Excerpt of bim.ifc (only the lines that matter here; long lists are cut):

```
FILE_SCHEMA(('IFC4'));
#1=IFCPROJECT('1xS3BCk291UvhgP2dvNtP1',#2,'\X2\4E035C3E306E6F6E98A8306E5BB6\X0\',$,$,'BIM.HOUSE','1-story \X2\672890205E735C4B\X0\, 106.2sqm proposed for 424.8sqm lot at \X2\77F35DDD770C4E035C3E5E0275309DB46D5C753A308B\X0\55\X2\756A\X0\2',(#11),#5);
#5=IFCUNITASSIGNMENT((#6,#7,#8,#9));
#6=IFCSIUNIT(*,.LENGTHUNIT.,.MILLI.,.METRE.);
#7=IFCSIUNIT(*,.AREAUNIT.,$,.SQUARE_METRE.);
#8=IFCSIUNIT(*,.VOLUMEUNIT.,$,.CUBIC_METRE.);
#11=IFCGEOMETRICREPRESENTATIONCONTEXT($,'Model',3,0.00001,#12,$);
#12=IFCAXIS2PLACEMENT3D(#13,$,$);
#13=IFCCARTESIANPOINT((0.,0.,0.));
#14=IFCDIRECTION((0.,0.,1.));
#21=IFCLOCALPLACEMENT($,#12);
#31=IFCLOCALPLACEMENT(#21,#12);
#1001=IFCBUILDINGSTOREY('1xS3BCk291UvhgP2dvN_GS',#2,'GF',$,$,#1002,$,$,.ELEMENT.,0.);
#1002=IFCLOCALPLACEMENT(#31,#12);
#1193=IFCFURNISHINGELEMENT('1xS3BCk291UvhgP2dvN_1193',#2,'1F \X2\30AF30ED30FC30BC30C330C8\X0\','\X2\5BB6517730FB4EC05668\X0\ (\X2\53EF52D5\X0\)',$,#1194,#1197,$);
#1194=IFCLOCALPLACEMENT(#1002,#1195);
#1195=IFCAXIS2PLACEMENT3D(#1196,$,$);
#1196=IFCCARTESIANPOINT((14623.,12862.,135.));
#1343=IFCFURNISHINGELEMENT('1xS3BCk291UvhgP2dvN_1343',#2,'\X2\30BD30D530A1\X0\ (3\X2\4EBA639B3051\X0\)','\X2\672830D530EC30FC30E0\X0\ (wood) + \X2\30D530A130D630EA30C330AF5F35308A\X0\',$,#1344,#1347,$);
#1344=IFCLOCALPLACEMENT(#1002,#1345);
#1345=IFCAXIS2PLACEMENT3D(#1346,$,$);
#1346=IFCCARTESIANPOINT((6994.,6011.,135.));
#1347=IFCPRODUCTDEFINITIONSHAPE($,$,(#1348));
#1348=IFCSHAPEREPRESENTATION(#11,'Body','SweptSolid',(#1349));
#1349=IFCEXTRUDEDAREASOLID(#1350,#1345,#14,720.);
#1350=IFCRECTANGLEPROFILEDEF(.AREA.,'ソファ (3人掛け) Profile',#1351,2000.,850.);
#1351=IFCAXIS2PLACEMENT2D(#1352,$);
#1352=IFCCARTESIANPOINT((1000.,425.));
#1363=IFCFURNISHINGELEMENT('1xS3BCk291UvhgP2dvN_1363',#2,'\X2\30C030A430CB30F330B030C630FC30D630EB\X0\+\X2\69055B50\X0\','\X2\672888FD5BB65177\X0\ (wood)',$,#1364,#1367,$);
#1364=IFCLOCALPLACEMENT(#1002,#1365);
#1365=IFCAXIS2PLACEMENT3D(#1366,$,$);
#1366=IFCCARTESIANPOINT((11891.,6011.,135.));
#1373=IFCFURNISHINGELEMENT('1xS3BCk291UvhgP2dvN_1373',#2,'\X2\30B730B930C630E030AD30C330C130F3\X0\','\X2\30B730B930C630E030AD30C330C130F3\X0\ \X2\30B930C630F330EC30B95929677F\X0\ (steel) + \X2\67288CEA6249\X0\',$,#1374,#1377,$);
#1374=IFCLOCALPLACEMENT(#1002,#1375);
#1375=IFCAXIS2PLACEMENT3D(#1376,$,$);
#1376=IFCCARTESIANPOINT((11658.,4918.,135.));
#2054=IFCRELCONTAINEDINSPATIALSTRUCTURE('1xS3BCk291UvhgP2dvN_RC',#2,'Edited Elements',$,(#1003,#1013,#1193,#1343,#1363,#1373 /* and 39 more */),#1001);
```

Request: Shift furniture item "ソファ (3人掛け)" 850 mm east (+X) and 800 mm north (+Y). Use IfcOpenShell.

```python
import ifcopenshell
import ifcopenshell.api.geometry
import ifcopenshell.util.placement

model = ifcopenshell.open("bim.ifc")

item = model.by_id(1343)
matrix = ifcopenshell.util.placement.get_local_placement(item.ObjectPlacement)
matrix[0, 3] += 850.0
matrix[1, 3] += 800.0
ifcopenshell.api.geometry.edit_object_placement(model, product=item, matrix=matrix, is_si=False)

print(ifcopenshell.util.placement.get_local_placement(item.ObjectPlacement).round(3) + 0.0)

model.write("bim_edited.ifc")
```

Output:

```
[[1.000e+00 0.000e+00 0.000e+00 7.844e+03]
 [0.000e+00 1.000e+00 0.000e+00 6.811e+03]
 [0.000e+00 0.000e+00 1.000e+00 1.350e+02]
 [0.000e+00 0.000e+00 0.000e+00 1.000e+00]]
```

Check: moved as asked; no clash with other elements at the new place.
